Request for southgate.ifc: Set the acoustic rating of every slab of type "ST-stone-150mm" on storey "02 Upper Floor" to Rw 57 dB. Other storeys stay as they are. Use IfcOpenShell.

First a look at what the model holds.

```python
import ifcopenshell
import ifcopenshell.util.element

model = ifcopenshell.open("southgate.ifc")
print(model.schema)
storey = next(s for s in model.by_type("IfcBuildingStorey") if s.Name == "02 Upper Floor")
slabs = [e for e in ifcopenshell.util.element.get_decomposition(storey) if e.is_a("IfcSlab")]
seen = {}
for e in slabs:
    element_type = ifcopenshell.util.element.get_type(e)
    key = (element_type.Name if element_type != e and element_type else None, ifcopenshell.util.element.get_pset(e, "Pset_SlabCommon", "AcousticRating"))
    seen[key] = seen.get(key, 0) + 1
for (name, value), count in sorted(seen.items(), key=str):
    print(count, "x", name, "|", value)
```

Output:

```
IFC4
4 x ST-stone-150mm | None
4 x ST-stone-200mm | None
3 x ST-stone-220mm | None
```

```python
import ifcopenshell
import ifcopenshell.api.pset
import ifcopenshell.util.element

model = ifcopenshell.open("southgate.ifc")

storey = next(s for s in model.by_type("IfcBuildingStorey") if s.Name == "02 Upper Floor")
slabs = [e for e in ifcopenshell.util.element.get_decomposition(storey) if e.is_a("IfcSlab")]

count = 0
for e in slabs:
    element_type = ifcopenshell.util.element.get_type(e)
    if element_type in (None, e) or element_type.Name != "ST-stone-150mm":
        continue
    # add_pset returns the element's existing set when there is one.
    pset = ifcopenshell.api.pset.add_pset(model, product=e, name="Pset_SlabCommon")
    ifcopenshell.api.pset.edit_pset(model, pset=pset, properties={"AcousticRating": "Rw 57 dB"})
    count += 1

print(count, "slabs updated")

model.write("southgate_v2.ifc")
```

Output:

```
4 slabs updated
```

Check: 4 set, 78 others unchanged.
